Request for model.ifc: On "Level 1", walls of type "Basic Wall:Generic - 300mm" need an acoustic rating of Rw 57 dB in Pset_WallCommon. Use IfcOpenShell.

First a look at what the model holds.

```python
import ifcopenshell
import ifcopenshell.util.element

model = ifcopenshell.open("model.ifc")
print(model.schema)
storey = next(s for s in model.by_type("IfcBuildingStorey") if s.Name == "Level 1")
walls = [e for e in ifcopenshell.util.element.get_decomposition(storey) if e.is_a("IfcWall")]
seen = {}
for e in walls:
    element_type = ifcopenshell.util.element.get_type(e)
    key = (element_type.Name if element_type != e and element_type else None, ifcopenshell.util.element.get_pset(e, "Pset_WallCommon", "AcousticRating"))
    seen[key] = seen.get(key, 0) + 1
for (name, value), count in sorted(seen.items(), key=str):
    print(count, "x", name, "|", value)
```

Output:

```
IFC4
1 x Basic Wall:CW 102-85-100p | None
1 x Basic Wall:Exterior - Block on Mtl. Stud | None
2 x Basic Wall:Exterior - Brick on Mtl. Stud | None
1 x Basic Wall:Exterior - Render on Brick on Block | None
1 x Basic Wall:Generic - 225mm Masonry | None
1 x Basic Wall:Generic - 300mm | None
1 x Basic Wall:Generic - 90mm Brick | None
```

```python
import ifcopenshell
import ifcopenshell.api.pset
import ifcopenshell.util.element

model = ifcopenshell.open("model.ifc")

storey = next(s for s in model.by_type("IfcBuildingStorey") if s.Name == "Level 1")
walls = [e for e in ifcopenshell.util.element.get_decomposition(storey) if e.is_a("IfcWall")]

count = 0
for e in walls:
    element_type = ifcopenshell.util.element.get_type(e)
    if element_type in (None, e) or element_type.Name != "Basic Wall:Generic - 300mm":
        continue
    # add_pset returns the element's existing set when there is one.
    pset = ifcopenshell.api.pset.add_pset(model, product=e, name="Pset_WallCommon")
    ifcopenshell.api.pset.edit_pset(model, pset=pset, properties={"AcousticRating": "Rw 57 dB"})
    count += 1

print(count, "walls updated")

model.write("model-out.ifc")
```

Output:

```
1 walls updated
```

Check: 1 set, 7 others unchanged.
